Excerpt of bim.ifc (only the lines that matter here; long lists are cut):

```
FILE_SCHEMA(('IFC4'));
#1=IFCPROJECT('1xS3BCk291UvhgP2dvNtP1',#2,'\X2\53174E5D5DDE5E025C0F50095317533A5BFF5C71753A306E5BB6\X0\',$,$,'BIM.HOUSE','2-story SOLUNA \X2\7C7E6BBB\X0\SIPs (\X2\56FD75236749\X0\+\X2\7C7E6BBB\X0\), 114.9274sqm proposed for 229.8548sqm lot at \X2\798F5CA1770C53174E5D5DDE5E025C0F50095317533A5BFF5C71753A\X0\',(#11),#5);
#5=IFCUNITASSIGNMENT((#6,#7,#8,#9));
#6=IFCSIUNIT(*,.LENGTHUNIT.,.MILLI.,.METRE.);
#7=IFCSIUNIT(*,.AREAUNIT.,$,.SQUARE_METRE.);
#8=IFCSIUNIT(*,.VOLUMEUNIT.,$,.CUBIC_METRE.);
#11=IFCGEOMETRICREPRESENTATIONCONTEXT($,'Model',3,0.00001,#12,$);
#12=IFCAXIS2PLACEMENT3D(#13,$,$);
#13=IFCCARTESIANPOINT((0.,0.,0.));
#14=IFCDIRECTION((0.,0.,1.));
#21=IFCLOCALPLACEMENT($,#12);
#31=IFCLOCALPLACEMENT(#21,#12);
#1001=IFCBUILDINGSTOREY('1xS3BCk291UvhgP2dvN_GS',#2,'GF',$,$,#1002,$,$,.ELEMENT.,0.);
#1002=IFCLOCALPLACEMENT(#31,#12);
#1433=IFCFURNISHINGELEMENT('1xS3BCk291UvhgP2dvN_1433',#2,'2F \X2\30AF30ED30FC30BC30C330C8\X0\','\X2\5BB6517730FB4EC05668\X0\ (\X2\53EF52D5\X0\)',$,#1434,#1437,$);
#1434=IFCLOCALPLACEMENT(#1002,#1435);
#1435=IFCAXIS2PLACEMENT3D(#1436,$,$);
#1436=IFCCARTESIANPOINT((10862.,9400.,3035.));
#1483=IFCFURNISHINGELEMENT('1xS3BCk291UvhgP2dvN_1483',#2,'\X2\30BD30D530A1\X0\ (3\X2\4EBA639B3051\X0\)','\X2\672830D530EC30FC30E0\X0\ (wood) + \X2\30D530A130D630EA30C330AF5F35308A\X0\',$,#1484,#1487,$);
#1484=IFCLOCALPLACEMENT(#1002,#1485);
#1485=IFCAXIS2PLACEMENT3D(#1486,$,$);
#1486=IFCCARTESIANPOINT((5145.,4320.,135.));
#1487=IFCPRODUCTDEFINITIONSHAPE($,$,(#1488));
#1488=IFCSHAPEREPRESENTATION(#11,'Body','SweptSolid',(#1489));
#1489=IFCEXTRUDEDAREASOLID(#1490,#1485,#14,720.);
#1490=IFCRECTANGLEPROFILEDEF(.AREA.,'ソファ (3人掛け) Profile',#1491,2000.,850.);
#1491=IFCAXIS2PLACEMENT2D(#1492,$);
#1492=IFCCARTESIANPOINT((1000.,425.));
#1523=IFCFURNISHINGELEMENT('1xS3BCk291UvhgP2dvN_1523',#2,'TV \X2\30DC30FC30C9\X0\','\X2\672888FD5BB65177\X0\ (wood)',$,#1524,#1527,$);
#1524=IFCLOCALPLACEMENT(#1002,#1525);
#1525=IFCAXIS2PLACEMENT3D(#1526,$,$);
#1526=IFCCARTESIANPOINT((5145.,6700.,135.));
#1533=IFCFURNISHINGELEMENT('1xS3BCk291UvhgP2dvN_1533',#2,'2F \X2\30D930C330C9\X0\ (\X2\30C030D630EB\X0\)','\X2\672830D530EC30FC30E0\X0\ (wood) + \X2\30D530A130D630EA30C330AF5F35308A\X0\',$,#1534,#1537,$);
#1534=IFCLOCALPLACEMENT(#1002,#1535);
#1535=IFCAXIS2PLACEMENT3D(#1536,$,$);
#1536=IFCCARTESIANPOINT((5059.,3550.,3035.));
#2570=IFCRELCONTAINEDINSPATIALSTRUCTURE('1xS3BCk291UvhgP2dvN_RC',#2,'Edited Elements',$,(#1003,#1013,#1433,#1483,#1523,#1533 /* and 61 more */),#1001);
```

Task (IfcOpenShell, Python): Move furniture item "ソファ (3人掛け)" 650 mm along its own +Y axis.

```python
import ifcopenshell
import ifcopenshell.api.geometry
import ifcopenshell.util.placement
import ifcopenshell.util.unit

model = ifcopenshell.open("bim.ifc")
unit_scale = ifcopenshell.util.unit.calculate_unit_scale(model)

item = model.by_id(1483)
matrix = ifcopenshell.util.placement.get_local_placement(item.ObjectPlacement)
matrix[:3, 3] += matrix[:3, 1] * 0.65 / unit_scale
ifcopenshell.api.geometry.edit_object_placement(model, product=item, matrix=matrix, is_si=False)

print(ifcopenshell.util.placement.get_local_placement(item.ObjectPlacement).round(3) + 0.0)

model.write("bim_edited.ifc")
```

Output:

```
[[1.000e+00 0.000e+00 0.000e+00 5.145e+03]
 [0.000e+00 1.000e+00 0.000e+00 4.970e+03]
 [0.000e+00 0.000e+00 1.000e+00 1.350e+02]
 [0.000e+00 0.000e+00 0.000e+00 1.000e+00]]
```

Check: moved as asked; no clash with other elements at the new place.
